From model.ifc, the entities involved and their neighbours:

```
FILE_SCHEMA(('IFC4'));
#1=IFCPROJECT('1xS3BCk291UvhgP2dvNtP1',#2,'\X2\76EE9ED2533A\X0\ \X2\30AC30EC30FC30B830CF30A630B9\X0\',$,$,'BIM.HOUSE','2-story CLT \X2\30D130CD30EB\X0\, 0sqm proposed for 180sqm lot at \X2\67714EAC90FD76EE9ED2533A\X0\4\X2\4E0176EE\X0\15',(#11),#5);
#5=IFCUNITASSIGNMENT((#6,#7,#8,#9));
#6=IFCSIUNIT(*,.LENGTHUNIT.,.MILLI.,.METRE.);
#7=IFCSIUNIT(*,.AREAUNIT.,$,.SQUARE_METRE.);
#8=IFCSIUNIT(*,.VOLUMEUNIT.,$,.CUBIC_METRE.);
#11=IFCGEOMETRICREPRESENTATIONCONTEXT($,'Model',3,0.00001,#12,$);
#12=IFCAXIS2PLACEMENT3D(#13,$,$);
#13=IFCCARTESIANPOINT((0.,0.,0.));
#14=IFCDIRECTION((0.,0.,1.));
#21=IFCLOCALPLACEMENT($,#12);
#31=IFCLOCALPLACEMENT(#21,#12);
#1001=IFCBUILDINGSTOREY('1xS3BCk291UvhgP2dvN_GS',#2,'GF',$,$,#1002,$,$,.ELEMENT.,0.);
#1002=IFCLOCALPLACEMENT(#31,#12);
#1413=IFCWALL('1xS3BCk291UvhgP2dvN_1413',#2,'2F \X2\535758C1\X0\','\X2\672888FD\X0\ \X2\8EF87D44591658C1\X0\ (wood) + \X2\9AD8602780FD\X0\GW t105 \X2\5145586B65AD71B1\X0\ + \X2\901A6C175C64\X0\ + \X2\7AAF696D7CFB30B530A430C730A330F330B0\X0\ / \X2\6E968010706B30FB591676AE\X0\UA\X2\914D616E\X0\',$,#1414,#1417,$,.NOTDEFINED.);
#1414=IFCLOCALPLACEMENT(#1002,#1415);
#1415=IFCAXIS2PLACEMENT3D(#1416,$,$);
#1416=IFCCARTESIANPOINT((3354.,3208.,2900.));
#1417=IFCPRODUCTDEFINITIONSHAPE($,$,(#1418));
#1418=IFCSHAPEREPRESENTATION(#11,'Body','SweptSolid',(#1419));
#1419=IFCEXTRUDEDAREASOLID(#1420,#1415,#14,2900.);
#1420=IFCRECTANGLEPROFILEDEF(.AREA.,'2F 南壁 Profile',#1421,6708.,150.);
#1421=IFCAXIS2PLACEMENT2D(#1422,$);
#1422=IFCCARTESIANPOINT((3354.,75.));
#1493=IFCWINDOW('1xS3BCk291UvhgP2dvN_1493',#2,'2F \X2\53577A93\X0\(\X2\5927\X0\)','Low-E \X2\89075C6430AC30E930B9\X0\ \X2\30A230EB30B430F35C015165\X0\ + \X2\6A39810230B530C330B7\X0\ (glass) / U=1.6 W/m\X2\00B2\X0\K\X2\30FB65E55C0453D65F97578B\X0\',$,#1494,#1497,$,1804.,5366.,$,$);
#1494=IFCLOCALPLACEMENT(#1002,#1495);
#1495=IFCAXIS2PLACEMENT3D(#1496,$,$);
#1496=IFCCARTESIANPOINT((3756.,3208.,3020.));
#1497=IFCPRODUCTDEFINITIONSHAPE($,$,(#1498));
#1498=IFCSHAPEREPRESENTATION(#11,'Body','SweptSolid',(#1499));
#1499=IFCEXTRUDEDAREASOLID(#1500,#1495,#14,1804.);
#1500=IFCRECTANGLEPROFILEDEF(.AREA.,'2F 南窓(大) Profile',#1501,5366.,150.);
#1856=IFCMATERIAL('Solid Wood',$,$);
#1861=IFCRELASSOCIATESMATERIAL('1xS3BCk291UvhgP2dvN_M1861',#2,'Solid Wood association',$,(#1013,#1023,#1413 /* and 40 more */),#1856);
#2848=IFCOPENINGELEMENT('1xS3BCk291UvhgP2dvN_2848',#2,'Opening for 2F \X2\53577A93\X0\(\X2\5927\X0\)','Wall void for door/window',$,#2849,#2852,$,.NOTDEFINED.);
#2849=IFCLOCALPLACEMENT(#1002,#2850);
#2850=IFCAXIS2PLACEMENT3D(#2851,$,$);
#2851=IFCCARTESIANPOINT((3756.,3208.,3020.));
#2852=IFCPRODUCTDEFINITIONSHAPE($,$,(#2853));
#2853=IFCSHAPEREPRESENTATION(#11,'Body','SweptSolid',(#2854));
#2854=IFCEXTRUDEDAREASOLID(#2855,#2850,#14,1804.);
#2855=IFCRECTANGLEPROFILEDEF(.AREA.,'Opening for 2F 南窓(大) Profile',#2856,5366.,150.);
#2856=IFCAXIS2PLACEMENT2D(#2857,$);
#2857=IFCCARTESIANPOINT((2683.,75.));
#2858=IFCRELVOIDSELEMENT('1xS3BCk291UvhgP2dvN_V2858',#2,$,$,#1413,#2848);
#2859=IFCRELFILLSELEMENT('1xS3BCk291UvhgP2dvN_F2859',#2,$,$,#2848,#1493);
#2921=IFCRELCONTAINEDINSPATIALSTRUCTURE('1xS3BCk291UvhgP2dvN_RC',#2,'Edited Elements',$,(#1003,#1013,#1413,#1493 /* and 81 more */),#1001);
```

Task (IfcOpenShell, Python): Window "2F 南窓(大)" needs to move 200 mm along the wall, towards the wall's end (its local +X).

```python
import ifcopenshell
import ifcopenshell.api.geometry
import ifcopenshell.util.placement
import ifcopenshell.util.unit

model = ifcopenshell.open("model.ifc")
unit_scale = ifcopenshell.util.unit.calculate_unit_scale(model)

window = model.by_guid("1xS3BCk291UvhgP2dvN_1493")
opening = window.FillsVoids[0].RelatingOpeningElement
wall = opening.VoidsElements[0].RelatingBuildingElement

wall_matrix = ifcopenshell.util.placement.get_local_placement(wall.ObjectPlacement)
shift = wall_matrix[:3, 0] * 0.2 / unit_scale
before = ifcopenshell.util.placement.get_local_placement(window.ObjectPlacement)[:3, 3].copy()

# The window is not placed relative to its opening, so move both.
for product in (opening, window):
    matrix = ifcopenshell.util.placement.get_local_placement(product.ObjectPlacement)
    matrix[:3, 3] += shift
    ifcopenshell.api.geometry.edit_object_placement(model, product=product, matrix=matrix, is_si=False)

after = ifcopenshell.util.placement.get_local_placement(window.ObjectPlacement)[:3, 3]
print("window moved by", (after - before).round(3) + 0.0)

model.write("model_edited.ifc")
```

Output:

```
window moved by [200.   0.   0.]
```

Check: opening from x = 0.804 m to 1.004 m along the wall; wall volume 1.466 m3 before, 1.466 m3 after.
